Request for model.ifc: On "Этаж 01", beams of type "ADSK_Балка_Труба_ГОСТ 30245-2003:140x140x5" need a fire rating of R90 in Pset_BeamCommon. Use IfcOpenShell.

First a look at what the model holds.

```python
import ifcopenshell
import ifcopenshell.util.element

model = ifcopenshell.open("model.ifc")
print(model.schema)
storey = next(s for s in model.by_type("IfcBuildingStorey") if s.Name == "Этаж 01")
beams = [e for e in ifcopenshell.util.element.get_decomposition(storey) if e.is_a("IfcBeam")]
seen = {}
for e in beams:
    element_type = ifcopenshell.util.element.get_type(e)
    key = (element_type.Name if element_type != e and element_type else None, ifcopenshell.util.element.get_pset(e, "Pset_BeamCommon", "FireRating"))
    seen[key] = seen.get(key, 0) + 1
for (name, value), count in sorted(seen.items(), key=str):
    print(count, "x", name, "|", value)
```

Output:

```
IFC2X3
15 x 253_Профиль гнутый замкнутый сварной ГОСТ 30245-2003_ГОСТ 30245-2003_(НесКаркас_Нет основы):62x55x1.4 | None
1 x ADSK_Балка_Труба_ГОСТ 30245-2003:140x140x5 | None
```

```python
import ifcopenshell
import ifcopenshell.api.pset
import ifcopenshell.util.element

model = ifcopenshell.open("model.ifc")

storey = next(s for s in model.by_type("IfcBuildingStorey") if s.Name == "Этаж 01")
beams = [e for e in ifcopenshell.util.element.get_decomposition(storey) if e.is_a("IfcBeam")]

count = 0
for e in beams:
    element_type = ifcopenshell.util.element.get_type(e)
    if element_type in (None, e) or element_type.Name != "ADSK_Балка_Труба_ГОСТ 30245-2003:140x140x5":
        continue
    # add_pset returns the element's existing set when there is one.
    pset = ifcopenshell.api.pset.add_pset(model, product=e, name="Pset_BeamCommon")
    ifcopenshell.api.pset.edit_pset(model, pset=pset, properties={"FireRating": "R90"})
    count += 1

print(count, "beams updated")

model.write("model_edited.ifc")
```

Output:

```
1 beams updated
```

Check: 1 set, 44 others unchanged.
